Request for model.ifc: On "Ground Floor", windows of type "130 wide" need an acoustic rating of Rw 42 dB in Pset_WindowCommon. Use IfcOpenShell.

First a look at what the model holds.

```python
import ifcopenshell
import ifcopenshell.util.element

model = ifcopenshell.open("model.ifc")
print(model.schema)
storey = next(s for s in model.by_type("IfcBuildingStorey") if s.Name == "Ground Floor")
windows = [e for e in ifcopenshell.util.element.get_decomposition(storey) if e.is_a("IfcWindow")]
seen = {}
for e in windows:
    element_type = ifcopenshell.util.element.get_type(e)
    key = (element_type.Name if element_type != e and element_type else None, ifcopenshell.util.element.get_pset(e, "Pset_WindowCommon", "AcousticRating"))
    seen[key] = seen.get(key, 0) + 1
for (name, value), count in sorted(seen.items(), key=str):
    print(count, "x", name, "|", value)
```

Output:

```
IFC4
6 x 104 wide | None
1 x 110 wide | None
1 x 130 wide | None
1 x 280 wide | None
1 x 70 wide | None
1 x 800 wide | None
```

```python
import ifcopenshell
import ifcopenshell.api.pset
import ifcopenshell.util.element

model = ifcopenshell.open("model.ifc")

storey = next(s for s in model.by_type("IfcBuildingStorey") if s.Name == "Ground Floor")
windows = [e for e in ifcopenshell.util.element.get_decomposition(storey) if e.is_a("IfcWindow")]

count = 0
for e in windows:
    element_type = ifcopenshell.util.element.get_type(e)
    if element_type in (None, e) or element_type.Name != "130 wide":
        continue
    # add_pset returns the element's existing set when there is one.
    pset = ifcopenshell.api.pset.add_pset(model, product=e, name="Pset_WindowCommon")
    ifcopenshell.api.pset.edit_pset(model, pset=pset, properties={"AcousticRating": "Rw 42 dB"})
    count += 1

print(count, "windows updated")

model.write("model_edited.ifc")
```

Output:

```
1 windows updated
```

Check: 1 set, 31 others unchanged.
